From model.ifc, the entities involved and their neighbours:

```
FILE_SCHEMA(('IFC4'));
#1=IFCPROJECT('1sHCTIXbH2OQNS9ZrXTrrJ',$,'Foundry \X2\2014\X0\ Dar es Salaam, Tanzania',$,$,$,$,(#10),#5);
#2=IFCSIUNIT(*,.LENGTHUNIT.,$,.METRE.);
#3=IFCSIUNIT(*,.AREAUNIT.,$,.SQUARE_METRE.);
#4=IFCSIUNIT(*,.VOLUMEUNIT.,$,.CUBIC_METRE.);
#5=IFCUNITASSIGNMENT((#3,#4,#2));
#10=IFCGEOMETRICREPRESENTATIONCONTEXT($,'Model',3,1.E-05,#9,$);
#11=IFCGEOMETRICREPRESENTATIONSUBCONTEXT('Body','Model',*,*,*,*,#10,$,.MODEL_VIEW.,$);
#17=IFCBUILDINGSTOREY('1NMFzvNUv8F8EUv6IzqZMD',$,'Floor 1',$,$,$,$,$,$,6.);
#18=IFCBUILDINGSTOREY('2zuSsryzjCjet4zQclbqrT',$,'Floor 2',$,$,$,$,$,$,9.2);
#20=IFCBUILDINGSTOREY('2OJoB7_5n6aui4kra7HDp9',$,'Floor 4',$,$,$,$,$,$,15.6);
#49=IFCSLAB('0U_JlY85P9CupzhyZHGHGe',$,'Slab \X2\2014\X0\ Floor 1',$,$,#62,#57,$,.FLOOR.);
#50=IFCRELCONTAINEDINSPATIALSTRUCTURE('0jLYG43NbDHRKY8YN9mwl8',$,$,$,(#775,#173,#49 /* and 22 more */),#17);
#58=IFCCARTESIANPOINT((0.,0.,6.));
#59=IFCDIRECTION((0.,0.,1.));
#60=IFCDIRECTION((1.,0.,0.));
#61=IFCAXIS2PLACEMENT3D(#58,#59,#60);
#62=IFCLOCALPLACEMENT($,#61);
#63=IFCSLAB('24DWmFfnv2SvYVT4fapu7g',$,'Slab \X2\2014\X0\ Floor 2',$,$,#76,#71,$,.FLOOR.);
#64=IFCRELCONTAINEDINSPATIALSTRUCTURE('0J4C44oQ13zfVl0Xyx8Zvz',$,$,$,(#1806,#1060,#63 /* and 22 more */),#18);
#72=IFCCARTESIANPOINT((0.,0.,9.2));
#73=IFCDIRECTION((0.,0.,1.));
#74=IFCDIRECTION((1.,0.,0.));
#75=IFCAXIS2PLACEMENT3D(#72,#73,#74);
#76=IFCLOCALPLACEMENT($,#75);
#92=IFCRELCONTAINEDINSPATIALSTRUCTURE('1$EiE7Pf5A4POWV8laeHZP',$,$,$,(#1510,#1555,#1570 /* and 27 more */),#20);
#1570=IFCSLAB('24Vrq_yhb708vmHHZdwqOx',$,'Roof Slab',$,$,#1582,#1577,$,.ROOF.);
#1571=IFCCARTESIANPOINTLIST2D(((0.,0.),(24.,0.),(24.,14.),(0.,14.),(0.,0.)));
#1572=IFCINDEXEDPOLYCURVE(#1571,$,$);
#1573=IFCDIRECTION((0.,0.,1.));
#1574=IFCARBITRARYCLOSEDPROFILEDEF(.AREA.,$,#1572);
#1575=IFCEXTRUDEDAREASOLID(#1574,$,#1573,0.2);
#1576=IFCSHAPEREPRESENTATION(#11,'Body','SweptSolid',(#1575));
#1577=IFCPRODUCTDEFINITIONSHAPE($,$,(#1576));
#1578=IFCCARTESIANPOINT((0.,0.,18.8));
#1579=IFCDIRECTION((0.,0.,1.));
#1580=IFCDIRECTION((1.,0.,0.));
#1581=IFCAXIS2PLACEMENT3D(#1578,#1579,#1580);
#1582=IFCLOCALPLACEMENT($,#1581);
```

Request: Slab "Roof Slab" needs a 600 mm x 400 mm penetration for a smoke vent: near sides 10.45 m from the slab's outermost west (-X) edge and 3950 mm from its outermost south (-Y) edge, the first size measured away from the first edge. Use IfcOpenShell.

```python
import numpy as np
import ifcopenshell
import ifcopenshell.api.feature
import ifcopenshell.api.geometry
import ifcopenshell.api.root
import ifcopenshell.geom
import ifcopenshell.util.placement
import ifcopenshell.util.representation
import ifcopenshell.util.shape
import ifcopenshell.util.unit

model = ifcopenshell.open("model.ifc")
unit_scale = ifcopenshell.util.unit.calculate_unit_scale(model)
settings = ifcopenshell.geom.settings()


def volume(element):
    """Net volume in cubic metres, openings subtracted."""
    shape = ifcopenshell.geom.create_shape(settings, element)
    return ifcopenshell.util.shape.get_volume(shape.geometry)


slab = model.by_guid("24Vrq_yhb708vmHHZdwqOx")
before = volume(slab)

# Extent in the slab's own axes, in metres. The edges named are its -X and -Y sides.
slab_shape = ifcopenshell.geom.create_shape(settings, slab)
vertices = ifcopenshell.util.shape.get_vertices(slab_shape.geometry)
x_min, y_min, bottom = vertices.min(axis=0)
top = vertices[:, 2].max()

opening = ifcopenshell.api.root.create_entity(model, ifc_class="IfcOpeningElement", name="Smoke vent opening", predefined_type="OPENING")
context = ifcopenshell.util.representation.get_context(model, "Model", "Body", "MODEL_VIEW")
width, depth = 0.6, 0.4
outline = [(0.0, 0.0), (width, 0.0), (width, depth), (0.0, depth), (0.0, 0.0)]
# Overshoot both faces by 50 mm so the cut is clean.
shape = ifcopenshell.api.geometry.add_slab_representation(
    model, context=context, depth=top - bottom + 0.1, polyline=outline
)
ifcopenshell.api.geometry.assign_representation(model, product=opening, representation=shape)

matrix = ifcopenshell.util.placement.get_local_placement(slab.ObjectPlacement)
matrix[:, 3] = matrix @ np.append(np.array([x_min + 10.45, y_min + 3.95, bottom - 0.05]) / unit_scale, 1.0)
ifcopenshell.api.geometry.edit_object_placement(model, product=opening, matrix=matrix, is_si=False)
ifcopenshell.api.feature.add_feature(model, feature=opening, element=slab)

after = volume(slab)

print(f"slab volume {before:.3f} -> {after:.3f} m3")

model.write("model-out.ifc")
```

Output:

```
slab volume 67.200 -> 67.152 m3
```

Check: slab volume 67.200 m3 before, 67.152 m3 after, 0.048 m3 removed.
